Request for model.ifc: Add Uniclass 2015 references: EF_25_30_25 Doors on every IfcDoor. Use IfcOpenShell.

First a look at what the model holds.

```python
import ifcopenshell

model = ifcopenshell.open("model.ifc")
print(model.schema)
print("classifications:", [c.Name for c in model.by_type("IfcClassification")])
for ifc_class in ("IfcDoor", "IfcRoof", "IfcStair", "IfcWall", "IfcWindow"):
    print(ifc_class, len(model.by_type(ifc_class)))
```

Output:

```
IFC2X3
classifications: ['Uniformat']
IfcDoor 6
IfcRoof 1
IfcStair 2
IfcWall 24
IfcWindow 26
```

```python
import ifcopenshell
import ifcopenshell.api.classification

model = ifcopenshell.open("model.ifc")

# IFC2X3 requires Source and Edition and has no link from the project to the system.
system = model.create_entity("IfcClassification", Source="NBS", Edition="2015", Name="Uniclass 2015")

codes = {
    "IfcDoor": ("EF_25_30_25", "Doors"),
}
for ifc_class, (code, name) in codes.items():
    products = model.by_type(ifc_class)
    ifcopenshell.api.classification.add_reference(
        model, products=products, classification=system, identification=code, name=name
    )
    print(code, len(products))

model.write("model_rev.ifc")
```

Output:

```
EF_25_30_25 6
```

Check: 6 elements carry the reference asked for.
